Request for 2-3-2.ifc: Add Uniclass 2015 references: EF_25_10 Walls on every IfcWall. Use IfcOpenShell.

First a look at what the model holds.

```python
import ifcopenshell

model = ifcopenshell.open("2-3-2.ifc")
print(model.schema)
print("classifications:", [c.Name for c in model.by_type("IfcClassification")])
for ifc_class in ("IfcDoor", "IfcRoof", "IfcStair", "IfcWall", "IfcWindow"):
    print(ifc_class, len(model.by_type(ifc_class)))
```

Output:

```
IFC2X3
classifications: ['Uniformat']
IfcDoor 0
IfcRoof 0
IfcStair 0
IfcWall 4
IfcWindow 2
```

```python
import ifcopenshell
import ifcopenshell.api.classification

model = ifcopenshell.open("2-3-2.ifc")

# IFC2X3 requires Source and Edition and has no link from the project to the system.
system = model.create_entity("IfcClassification", Source="NBS", Edition="2015", Name="Uniclass 2015")

codes = {
    "IfcWall": ("EF_25_10", "Walls"),
}
for ifc_class, (code, name) in codes.items():
    products = model.by_type(ifc_class)
    ifcopenshell.api.classification.add_reference(
        model, products=products, classification=system, identification=code, name=name
    )
    print(code, len(products))

model.write("2-3-2_v2.ifc")
```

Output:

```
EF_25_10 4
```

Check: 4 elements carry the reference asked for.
